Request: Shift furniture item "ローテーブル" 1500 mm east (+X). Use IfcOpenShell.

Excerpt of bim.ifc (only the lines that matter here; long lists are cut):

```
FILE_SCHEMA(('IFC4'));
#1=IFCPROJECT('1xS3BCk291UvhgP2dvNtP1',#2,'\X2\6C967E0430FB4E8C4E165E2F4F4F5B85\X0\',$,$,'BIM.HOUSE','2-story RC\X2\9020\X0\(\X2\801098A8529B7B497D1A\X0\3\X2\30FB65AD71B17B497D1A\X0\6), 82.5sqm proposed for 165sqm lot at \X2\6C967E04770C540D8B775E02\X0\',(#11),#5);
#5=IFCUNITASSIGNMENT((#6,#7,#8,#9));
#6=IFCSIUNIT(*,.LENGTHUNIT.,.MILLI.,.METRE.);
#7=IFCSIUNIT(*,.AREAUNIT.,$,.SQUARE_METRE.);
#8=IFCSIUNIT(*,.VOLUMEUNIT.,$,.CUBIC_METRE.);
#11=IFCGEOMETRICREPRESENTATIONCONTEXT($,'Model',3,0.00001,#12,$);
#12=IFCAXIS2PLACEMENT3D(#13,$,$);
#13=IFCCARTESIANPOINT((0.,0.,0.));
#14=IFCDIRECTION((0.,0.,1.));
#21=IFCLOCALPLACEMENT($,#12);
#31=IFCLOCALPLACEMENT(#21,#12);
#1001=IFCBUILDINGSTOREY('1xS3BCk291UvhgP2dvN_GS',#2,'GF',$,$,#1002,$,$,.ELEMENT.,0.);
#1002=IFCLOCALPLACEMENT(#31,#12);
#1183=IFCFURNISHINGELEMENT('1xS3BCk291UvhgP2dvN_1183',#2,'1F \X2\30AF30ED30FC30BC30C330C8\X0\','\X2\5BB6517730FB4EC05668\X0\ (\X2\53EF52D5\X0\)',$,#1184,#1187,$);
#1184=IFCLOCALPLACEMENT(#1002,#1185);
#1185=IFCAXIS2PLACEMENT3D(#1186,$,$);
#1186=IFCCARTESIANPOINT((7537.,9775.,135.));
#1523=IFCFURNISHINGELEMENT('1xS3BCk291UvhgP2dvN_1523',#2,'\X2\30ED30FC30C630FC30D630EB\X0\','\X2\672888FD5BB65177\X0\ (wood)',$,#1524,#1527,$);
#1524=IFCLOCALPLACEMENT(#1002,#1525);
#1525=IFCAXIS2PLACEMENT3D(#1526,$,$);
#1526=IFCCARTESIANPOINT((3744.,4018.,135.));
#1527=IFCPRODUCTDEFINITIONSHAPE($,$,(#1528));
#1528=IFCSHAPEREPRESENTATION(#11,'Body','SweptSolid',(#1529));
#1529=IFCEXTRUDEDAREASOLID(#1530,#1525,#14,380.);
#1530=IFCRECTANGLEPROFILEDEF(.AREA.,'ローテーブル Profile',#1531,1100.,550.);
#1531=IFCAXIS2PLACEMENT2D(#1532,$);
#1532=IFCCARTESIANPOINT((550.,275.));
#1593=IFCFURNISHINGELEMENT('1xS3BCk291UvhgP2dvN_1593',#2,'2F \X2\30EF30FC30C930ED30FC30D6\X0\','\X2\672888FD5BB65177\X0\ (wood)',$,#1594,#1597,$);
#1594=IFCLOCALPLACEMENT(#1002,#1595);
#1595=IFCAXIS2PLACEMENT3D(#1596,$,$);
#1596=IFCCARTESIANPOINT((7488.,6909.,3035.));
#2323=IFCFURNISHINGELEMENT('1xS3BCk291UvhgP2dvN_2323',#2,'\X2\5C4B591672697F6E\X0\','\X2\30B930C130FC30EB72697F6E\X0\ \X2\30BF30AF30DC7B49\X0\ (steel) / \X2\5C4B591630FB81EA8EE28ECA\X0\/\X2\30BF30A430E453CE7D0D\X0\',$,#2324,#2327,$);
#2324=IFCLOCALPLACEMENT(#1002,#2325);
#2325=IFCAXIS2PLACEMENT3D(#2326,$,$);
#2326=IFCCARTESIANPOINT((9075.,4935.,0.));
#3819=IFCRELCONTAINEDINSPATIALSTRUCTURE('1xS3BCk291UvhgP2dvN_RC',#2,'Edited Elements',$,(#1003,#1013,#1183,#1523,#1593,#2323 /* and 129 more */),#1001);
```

```python
import ifcopenshell
import ifcopenshell.api.geometry
import ifcopenshell.util.placement

model = ifcopenshell.open("bim.ifc")

item = model.by_guid("1xS3BCk291UvhgP2dvN_1523")
matrix = ifcopenshell.util.placement.get_local_placement(item.ObjectPlacement)
matrix[0, 3] += 1500.0
ifcopenshell.api.geometry.edit_object_placement(model, product=item, matrix=matrix, is_si=False)

print(ifcopenshell.util.placement.get_local_placement(item.ObjectPlacement).round(3) + 0.0)

model.write("bim_rev.ifc")
```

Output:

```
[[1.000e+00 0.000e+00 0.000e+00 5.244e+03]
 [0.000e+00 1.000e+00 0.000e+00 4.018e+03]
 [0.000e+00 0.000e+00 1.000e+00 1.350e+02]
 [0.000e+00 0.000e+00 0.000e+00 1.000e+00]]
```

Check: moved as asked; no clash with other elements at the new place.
